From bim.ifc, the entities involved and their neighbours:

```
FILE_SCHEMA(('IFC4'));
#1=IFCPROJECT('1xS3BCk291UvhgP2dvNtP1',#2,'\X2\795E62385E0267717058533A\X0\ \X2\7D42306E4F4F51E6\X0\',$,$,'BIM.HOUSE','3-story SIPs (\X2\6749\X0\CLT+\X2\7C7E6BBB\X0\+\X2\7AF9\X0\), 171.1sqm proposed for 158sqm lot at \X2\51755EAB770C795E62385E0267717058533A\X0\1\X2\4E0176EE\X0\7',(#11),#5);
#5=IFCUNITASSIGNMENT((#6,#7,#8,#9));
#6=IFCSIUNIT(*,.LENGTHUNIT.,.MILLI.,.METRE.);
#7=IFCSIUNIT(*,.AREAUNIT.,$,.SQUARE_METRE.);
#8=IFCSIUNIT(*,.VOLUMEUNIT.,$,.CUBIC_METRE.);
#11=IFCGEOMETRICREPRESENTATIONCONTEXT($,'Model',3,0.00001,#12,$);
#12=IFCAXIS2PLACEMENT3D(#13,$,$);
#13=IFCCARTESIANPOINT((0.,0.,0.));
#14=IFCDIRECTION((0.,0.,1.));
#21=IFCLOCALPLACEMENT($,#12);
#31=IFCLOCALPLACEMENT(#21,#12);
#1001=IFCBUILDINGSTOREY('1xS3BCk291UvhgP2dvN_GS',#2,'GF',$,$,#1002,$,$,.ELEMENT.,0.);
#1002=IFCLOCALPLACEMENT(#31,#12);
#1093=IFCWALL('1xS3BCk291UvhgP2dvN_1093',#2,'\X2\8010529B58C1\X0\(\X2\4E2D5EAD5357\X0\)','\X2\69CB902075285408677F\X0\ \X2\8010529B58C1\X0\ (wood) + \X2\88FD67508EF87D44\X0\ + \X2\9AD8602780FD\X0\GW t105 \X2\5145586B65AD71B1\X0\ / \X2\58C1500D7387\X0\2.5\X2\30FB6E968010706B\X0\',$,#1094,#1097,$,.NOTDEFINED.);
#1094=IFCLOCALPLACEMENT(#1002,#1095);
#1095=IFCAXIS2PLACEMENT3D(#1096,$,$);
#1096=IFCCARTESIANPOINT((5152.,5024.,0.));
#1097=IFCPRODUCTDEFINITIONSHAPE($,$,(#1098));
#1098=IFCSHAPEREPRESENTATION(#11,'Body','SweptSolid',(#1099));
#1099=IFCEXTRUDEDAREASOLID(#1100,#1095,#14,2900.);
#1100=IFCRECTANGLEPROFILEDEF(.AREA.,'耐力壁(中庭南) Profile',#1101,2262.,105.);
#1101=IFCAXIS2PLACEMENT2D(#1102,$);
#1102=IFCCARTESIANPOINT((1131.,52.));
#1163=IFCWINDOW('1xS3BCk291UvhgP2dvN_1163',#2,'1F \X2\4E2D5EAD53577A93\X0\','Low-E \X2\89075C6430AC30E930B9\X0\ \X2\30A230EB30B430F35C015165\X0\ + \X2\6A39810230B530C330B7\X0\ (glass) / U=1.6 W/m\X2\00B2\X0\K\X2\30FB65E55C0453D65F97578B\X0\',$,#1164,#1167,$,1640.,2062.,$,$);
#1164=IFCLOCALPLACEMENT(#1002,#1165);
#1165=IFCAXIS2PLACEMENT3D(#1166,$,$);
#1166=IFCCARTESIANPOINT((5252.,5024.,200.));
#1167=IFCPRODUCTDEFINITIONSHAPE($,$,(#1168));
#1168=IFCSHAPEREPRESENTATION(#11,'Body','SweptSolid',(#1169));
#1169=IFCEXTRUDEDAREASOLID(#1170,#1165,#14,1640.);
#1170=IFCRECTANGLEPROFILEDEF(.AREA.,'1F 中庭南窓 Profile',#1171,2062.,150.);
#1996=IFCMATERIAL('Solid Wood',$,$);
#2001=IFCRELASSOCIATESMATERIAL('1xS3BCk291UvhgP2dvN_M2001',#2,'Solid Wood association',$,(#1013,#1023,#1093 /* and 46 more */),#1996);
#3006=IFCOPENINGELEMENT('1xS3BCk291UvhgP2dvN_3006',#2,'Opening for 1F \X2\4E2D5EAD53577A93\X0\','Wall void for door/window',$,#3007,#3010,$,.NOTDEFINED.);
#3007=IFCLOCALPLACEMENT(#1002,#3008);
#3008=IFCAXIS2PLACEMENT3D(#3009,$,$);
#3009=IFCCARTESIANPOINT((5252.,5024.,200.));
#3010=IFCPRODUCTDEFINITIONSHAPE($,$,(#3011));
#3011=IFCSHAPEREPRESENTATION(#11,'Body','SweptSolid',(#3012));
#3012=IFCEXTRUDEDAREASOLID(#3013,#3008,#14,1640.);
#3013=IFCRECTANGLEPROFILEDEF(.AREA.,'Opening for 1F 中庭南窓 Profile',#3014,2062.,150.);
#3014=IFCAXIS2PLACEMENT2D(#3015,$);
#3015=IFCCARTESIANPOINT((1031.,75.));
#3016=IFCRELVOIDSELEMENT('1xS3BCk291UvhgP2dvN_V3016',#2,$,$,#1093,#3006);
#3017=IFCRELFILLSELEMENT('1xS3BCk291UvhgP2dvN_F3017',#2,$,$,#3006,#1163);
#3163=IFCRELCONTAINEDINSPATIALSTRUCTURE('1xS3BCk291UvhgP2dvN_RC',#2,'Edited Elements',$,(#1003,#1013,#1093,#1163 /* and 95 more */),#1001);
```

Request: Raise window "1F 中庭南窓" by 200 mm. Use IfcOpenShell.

```python
import numpy as np
import ifcopenshell
import ifcopenshell.api.geometry
import ifcopenshell.util.placement
import ifcopenshell.util.unit

model = ifcopenshell.open("bim.ifc")
unit_scale = ifcopenshell.util.unit.calculate_unit_scale(model)

window = model.by_guid("1xS3BCk291UvhgP2dvN_1163")
opening = window.FillsVoids[0].RelatingOpeningElement
dz = 0.2 / unit_scale

shift = np.array([0.0, 0.0, dz])
# The window is not placed relative to its opening, so move both.
for product in (opening, window):
    matrix = ifcopenshell.util.placement.get_local_placement(product.ObjectPlacement)
    matrix[:3, 3] += shift
    ifcopenshell.api.geometry.edit_object_placement(model, product=product, matrix=matrix, is_si=False)

print(f"moved by {dz * unit_scale:+.3f} m")

model.write("bim-out.ifc")
```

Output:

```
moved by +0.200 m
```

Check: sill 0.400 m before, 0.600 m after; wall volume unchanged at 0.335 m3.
